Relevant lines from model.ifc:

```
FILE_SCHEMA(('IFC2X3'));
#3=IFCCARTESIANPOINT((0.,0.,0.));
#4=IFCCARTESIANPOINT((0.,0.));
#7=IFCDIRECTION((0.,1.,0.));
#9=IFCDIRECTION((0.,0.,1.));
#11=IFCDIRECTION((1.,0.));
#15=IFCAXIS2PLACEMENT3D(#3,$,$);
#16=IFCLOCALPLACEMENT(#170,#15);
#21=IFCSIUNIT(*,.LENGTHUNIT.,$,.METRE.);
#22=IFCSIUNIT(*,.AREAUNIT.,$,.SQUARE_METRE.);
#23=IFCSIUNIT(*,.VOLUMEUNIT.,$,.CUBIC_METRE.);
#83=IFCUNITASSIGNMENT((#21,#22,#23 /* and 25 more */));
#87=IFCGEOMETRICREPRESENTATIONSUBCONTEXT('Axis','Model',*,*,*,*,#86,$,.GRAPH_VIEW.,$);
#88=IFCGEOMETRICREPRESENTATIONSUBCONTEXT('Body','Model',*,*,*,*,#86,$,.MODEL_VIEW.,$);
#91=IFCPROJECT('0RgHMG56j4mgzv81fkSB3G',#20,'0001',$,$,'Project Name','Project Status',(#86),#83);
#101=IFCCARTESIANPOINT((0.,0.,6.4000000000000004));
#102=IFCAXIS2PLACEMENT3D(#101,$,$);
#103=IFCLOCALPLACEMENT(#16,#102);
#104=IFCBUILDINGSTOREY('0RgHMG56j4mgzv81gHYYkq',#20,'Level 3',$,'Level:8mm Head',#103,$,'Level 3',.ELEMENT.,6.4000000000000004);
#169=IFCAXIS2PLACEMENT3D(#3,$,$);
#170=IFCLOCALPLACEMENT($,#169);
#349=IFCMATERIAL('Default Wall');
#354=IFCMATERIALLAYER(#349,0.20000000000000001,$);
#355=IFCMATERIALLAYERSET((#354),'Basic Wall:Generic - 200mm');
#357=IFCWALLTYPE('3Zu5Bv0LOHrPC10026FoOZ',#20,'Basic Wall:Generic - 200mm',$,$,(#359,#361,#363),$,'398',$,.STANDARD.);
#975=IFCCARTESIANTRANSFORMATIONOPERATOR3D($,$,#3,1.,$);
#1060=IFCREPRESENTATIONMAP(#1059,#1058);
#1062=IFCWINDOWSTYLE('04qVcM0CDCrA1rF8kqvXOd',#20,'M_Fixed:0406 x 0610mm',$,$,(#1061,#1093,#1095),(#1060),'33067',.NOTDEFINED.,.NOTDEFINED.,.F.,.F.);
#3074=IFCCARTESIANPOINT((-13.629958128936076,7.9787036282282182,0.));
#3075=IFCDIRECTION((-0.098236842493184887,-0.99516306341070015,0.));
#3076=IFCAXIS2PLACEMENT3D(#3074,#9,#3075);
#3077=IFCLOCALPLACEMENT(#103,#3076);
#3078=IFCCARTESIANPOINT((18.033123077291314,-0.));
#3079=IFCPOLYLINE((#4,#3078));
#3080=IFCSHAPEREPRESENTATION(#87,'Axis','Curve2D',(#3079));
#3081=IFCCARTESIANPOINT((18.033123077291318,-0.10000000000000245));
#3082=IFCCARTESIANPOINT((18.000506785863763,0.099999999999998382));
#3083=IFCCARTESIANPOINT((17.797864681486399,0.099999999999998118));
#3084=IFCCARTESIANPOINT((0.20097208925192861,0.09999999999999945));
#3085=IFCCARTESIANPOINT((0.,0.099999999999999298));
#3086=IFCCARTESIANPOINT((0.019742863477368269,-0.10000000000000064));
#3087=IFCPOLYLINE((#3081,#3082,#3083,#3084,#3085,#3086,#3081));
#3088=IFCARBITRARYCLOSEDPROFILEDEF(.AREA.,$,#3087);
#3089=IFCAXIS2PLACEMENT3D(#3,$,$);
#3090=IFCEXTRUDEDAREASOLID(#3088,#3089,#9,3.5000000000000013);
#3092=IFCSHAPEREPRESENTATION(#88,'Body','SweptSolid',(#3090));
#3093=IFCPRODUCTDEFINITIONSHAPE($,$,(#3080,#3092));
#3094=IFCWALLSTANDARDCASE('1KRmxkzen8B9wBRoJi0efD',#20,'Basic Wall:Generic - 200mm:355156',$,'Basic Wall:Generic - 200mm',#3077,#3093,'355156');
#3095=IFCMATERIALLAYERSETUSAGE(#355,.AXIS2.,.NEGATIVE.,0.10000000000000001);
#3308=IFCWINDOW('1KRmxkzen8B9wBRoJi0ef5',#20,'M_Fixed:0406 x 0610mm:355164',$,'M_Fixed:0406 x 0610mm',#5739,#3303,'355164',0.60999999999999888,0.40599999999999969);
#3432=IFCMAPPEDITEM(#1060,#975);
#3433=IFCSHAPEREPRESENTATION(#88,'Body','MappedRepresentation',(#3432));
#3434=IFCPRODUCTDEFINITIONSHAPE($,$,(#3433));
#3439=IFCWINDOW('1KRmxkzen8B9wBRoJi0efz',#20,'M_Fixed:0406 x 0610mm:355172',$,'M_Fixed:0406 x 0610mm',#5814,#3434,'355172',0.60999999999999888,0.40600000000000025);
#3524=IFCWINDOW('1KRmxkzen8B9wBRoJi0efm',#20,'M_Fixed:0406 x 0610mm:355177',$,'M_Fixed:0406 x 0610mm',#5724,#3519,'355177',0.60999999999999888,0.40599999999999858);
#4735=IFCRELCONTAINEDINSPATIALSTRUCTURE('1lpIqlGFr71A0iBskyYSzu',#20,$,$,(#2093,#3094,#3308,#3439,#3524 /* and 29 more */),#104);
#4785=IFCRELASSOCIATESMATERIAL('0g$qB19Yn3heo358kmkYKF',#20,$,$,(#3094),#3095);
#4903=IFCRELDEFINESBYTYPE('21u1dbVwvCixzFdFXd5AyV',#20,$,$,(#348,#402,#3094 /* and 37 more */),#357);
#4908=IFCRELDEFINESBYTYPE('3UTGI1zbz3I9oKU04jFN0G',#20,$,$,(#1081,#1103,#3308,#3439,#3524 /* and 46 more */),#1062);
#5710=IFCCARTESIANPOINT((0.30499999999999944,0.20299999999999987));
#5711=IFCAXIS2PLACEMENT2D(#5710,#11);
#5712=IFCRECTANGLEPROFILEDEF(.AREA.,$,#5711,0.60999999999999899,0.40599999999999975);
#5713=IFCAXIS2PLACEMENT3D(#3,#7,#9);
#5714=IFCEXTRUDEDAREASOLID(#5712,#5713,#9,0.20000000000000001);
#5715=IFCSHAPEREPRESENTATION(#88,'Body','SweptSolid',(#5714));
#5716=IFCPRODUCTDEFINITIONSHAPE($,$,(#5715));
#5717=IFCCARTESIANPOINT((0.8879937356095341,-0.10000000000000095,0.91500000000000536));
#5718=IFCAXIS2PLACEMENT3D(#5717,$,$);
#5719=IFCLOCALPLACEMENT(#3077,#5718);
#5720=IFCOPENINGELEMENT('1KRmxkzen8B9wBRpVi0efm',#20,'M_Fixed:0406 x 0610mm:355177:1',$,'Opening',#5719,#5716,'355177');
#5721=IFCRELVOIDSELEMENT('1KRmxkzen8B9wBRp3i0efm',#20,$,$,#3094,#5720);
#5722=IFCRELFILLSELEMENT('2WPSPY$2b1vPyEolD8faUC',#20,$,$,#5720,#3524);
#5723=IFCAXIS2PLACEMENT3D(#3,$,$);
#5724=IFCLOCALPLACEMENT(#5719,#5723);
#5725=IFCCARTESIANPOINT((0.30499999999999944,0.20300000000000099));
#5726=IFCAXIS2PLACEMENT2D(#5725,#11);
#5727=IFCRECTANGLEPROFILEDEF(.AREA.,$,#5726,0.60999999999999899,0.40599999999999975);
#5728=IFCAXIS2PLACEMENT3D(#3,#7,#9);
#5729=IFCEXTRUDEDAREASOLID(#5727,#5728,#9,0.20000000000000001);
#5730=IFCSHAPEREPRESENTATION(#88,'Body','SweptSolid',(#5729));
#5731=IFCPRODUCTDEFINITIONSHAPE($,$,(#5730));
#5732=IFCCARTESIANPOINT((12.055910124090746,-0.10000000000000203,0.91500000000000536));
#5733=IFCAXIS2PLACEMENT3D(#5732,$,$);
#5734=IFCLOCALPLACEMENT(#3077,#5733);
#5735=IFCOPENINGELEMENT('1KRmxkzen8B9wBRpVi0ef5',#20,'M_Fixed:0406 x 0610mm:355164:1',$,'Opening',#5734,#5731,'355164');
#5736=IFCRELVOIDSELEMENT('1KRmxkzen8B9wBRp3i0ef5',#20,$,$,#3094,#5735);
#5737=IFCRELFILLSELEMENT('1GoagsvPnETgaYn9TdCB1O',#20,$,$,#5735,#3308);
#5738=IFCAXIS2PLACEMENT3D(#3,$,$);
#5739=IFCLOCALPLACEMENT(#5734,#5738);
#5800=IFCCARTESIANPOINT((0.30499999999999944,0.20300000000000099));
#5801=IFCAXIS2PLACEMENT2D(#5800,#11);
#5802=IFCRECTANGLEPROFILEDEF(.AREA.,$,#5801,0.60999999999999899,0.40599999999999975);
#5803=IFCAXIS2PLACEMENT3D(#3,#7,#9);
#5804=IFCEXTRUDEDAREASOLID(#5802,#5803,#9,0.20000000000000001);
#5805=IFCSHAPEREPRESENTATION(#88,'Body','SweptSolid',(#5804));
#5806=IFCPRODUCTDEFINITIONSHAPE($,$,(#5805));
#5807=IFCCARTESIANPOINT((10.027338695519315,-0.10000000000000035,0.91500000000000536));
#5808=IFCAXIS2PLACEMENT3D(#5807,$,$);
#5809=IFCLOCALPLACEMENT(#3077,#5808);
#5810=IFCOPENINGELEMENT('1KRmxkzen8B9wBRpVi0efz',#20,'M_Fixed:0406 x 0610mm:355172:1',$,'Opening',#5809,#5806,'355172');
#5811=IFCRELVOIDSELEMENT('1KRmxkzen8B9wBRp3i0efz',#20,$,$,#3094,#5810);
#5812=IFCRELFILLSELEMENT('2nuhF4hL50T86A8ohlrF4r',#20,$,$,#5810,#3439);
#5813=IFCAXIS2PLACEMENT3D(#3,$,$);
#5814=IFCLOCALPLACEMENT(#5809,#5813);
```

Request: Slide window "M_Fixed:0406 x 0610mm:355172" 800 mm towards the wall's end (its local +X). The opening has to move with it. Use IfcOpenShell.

```python
import ifcopenshell
import ifcopenshell.api.geometry
import ifcopenshell.util.placement
import ifcopenshell.util.unit

model = ifcopenshell.open("model.ifc")
unit_scale = ifcopenshell.util.unit.calculate_unit_scale(model)

window = model.by_guid("1KRmxkzen8B9wBRoJi0efz")
opening = window.FillsVoids[0].RelatingOpeningElement
wall = opening.VoidsElements[0].RelatingBuildingElement

wall_matrix = ifcopenshell.util.placement.get_local_placement(wall.ObjectPlacement)
shift = wall_matrix[:3, 0] * 0.8 / unit_scale
before = ifcopenshell.util.placement.get_local_placement(window.ObjectPlacement)[:3, 3].copy()

# The window is placed relative to its opening, so it follows when the opening moves.
matrix = ifcopenshell.util.placement.get_local_placement(opening.ObjectPlacement)
matrix[:3, 3] += shift
ifcopenshell.api.geometry.edit_object_placement(
    model, product=opening, matrix=matrix, is_si=False, should_transform_children=True
)

after = ifcopenshell.util.placement.get_local_placement(window.ObjectPlacement)[:3, 3]
print("window moved by", (after - before).round(3) + 0.0)

model.write("model_rev.ifc")
```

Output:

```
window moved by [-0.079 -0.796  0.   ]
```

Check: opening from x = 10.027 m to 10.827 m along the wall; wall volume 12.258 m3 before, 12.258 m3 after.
